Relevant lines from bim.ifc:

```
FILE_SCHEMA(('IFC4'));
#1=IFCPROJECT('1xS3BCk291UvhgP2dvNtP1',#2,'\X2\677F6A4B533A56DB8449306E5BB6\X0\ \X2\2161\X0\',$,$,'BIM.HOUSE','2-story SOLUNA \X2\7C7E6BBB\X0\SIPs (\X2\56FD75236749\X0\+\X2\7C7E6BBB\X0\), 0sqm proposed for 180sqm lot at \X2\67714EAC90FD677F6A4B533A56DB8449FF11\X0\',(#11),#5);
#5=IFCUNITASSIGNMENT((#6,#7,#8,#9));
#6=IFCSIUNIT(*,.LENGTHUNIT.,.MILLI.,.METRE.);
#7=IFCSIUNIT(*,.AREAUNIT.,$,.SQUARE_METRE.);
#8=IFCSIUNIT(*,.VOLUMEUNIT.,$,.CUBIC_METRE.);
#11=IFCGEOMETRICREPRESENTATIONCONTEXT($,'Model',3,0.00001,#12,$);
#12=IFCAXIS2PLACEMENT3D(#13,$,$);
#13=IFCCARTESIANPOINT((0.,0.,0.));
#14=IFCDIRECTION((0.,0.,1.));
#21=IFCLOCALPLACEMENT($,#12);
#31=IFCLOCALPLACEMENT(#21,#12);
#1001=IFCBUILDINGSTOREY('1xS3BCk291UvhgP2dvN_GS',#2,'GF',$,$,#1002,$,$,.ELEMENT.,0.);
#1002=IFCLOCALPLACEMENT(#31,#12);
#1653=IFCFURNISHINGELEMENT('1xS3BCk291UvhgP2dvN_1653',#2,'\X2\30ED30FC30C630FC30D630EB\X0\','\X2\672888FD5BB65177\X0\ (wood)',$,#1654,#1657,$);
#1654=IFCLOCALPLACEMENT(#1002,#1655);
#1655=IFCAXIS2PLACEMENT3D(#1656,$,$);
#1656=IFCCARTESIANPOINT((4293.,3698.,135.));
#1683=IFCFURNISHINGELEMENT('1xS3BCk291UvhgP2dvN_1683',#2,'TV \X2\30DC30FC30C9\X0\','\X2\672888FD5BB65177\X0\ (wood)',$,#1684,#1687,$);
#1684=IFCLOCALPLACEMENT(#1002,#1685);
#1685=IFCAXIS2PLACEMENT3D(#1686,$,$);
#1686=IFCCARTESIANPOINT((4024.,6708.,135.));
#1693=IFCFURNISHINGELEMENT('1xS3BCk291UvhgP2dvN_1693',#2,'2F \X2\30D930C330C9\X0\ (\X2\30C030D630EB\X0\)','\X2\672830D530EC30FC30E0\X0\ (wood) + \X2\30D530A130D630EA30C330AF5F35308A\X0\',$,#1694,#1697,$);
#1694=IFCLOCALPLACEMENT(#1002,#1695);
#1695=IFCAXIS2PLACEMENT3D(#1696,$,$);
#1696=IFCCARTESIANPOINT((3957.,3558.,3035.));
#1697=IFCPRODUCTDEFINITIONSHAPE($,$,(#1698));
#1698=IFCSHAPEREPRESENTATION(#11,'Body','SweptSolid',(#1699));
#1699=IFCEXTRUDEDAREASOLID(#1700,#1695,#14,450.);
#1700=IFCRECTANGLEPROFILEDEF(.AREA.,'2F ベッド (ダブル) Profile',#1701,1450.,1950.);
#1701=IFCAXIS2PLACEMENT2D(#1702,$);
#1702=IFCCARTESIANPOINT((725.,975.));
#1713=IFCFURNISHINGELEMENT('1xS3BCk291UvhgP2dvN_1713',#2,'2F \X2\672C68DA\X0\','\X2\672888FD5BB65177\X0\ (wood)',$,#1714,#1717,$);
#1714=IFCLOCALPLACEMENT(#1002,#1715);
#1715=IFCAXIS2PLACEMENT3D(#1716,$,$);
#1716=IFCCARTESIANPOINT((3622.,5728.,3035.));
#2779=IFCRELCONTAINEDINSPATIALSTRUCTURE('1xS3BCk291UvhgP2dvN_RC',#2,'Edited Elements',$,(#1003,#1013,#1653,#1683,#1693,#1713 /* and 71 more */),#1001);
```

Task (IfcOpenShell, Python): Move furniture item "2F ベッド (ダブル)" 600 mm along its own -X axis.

```python
import ifcopenshell
import ifcopenshell.api.geometry
import ifcopenshell.util.placement

model = ifcopenshell.open("bim.ifc")

item = model.by_id(1693)
matrix = ifcopenshell.util.placement.get_local_placement(item.ObjectPlacement)
matrix[:3, 3] -= matrix[:3, 0] * 600.0
ifcopenshell.api.geometry.edit_object_placement(model, product=item, matrix=matrix, is_si=False)

print(ifcopenshell.util.placement.get_local_placement(item.ObjectPlacement).round(3) + 0.0)

model.write("bim_rev.ifc")
```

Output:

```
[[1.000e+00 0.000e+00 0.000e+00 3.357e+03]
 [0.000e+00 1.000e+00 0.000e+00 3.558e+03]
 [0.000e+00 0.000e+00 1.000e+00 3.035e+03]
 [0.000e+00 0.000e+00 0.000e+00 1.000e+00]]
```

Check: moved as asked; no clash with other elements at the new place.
